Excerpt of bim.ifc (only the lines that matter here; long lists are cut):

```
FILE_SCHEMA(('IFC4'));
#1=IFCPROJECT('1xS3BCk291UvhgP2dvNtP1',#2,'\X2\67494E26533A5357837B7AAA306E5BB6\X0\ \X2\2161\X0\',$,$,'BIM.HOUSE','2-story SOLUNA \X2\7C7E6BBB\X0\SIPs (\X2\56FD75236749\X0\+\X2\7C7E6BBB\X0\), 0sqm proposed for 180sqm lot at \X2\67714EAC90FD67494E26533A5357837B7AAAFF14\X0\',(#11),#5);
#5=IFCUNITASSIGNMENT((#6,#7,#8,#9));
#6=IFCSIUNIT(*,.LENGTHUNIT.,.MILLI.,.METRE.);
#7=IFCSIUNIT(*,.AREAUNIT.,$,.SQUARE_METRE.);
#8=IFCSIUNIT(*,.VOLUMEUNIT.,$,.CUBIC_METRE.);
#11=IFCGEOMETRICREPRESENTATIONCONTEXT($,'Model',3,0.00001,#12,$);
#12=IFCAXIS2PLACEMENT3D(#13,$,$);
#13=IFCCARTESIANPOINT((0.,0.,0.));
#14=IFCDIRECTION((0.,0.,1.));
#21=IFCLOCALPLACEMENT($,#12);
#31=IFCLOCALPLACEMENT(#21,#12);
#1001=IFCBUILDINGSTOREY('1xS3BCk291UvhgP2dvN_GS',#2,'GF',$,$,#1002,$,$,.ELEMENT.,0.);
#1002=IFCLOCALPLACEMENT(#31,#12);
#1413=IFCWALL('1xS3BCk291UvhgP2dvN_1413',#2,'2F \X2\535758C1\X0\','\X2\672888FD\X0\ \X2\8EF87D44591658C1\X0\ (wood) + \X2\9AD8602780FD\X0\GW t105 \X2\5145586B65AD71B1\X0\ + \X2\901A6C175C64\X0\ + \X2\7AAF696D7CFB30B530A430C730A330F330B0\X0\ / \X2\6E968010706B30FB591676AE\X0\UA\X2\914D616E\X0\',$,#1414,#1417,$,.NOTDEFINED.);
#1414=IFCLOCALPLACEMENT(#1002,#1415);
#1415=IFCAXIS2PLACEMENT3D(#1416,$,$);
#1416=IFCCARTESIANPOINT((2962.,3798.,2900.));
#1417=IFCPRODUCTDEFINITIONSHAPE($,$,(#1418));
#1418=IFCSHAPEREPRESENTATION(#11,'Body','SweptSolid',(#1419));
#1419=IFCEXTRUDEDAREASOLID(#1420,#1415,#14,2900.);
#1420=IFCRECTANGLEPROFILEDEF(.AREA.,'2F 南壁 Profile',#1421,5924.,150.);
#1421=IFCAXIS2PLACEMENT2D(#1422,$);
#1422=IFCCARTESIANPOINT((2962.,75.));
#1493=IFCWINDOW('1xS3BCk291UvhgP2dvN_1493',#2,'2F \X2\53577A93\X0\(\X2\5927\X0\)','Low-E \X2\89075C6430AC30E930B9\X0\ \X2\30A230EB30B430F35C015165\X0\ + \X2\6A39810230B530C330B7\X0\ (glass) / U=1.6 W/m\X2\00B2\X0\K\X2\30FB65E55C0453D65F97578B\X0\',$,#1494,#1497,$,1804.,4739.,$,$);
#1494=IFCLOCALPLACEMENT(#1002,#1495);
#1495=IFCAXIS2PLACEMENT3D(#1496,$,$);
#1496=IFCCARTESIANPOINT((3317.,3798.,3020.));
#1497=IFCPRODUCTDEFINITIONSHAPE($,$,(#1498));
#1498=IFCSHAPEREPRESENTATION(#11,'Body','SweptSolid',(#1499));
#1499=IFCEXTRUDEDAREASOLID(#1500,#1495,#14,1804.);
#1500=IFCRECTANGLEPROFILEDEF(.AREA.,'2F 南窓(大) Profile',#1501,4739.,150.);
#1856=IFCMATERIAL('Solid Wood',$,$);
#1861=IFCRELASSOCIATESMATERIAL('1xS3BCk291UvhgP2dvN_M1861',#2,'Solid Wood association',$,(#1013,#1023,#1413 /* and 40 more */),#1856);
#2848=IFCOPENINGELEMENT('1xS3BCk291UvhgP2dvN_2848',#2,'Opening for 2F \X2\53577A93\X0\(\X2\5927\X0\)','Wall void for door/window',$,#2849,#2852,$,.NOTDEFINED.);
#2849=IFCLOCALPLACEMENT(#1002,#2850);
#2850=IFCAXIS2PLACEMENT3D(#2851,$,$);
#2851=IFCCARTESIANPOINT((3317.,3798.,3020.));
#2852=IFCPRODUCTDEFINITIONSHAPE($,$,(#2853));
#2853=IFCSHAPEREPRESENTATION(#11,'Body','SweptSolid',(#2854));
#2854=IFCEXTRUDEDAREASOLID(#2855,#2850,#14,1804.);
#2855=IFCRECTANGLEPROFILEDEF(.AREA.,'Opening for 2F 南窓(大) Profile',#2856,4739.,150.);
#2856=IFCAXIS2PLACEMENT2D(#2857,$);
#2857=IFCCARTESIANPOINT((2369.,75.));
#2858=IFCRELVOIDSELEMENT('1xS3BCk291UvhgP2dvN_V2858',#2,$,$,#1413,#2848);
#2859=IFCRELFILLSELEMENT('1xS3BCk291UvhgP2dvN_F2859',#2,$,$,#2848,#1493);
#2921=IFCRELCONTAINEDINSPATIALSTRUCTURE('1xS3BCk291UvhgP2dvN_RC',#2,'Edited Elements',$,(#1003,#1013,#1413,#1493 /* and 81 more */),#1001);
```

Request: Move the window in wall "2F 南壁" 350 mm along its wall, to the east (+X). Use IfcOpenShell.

```python
import ifcopenshell
import ifcopenshell.api.geometry
import ifcopenshell.util.placement
import ifcopenshell.util.unit

model = ifcopenshell.open("bim.ifc")
unit_scale = ifcopenshell.util.unit.calculate_unit_scale(model)

window = model.by_id(1493)
opening = window.FillsVoids[0].RelatingOpeningElement
wall = opening.VoidsElements[0].RelatingBuildingElement

wall_matrix = ifcopenshell.util.placement.get_local_placement(wall.ObjectPlacement)
shift = wall_matrix[:3, 0] * 0.35 / unit_scale
before = ifcopenshell.util.placement.get_local_placement(window.ObjectPlacement)[:3, 3].copy()

# The window is not placed relative to its opening, so move both.
for product in (opening, window):
    matrix = ifcopenshell.util.placement.get_local_placement(product.ObjectPlacement)
    matrix[:3, 3] += shift
    ifcopenshell.api.geometry.edit_object_placement(model, product=product, matrix=matrix, is_si=False)

after = ifcopenshell.util.placement.get_local_placement(window.ObjectPlacement)[:3, 3]
print("window moved by", (after - before).round(3) + 0.0)

model.write("bim_edited.ifc")
```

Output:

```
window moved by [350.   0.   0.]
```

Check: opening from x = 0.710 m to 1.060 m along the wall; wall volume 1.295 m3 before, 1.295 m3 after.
